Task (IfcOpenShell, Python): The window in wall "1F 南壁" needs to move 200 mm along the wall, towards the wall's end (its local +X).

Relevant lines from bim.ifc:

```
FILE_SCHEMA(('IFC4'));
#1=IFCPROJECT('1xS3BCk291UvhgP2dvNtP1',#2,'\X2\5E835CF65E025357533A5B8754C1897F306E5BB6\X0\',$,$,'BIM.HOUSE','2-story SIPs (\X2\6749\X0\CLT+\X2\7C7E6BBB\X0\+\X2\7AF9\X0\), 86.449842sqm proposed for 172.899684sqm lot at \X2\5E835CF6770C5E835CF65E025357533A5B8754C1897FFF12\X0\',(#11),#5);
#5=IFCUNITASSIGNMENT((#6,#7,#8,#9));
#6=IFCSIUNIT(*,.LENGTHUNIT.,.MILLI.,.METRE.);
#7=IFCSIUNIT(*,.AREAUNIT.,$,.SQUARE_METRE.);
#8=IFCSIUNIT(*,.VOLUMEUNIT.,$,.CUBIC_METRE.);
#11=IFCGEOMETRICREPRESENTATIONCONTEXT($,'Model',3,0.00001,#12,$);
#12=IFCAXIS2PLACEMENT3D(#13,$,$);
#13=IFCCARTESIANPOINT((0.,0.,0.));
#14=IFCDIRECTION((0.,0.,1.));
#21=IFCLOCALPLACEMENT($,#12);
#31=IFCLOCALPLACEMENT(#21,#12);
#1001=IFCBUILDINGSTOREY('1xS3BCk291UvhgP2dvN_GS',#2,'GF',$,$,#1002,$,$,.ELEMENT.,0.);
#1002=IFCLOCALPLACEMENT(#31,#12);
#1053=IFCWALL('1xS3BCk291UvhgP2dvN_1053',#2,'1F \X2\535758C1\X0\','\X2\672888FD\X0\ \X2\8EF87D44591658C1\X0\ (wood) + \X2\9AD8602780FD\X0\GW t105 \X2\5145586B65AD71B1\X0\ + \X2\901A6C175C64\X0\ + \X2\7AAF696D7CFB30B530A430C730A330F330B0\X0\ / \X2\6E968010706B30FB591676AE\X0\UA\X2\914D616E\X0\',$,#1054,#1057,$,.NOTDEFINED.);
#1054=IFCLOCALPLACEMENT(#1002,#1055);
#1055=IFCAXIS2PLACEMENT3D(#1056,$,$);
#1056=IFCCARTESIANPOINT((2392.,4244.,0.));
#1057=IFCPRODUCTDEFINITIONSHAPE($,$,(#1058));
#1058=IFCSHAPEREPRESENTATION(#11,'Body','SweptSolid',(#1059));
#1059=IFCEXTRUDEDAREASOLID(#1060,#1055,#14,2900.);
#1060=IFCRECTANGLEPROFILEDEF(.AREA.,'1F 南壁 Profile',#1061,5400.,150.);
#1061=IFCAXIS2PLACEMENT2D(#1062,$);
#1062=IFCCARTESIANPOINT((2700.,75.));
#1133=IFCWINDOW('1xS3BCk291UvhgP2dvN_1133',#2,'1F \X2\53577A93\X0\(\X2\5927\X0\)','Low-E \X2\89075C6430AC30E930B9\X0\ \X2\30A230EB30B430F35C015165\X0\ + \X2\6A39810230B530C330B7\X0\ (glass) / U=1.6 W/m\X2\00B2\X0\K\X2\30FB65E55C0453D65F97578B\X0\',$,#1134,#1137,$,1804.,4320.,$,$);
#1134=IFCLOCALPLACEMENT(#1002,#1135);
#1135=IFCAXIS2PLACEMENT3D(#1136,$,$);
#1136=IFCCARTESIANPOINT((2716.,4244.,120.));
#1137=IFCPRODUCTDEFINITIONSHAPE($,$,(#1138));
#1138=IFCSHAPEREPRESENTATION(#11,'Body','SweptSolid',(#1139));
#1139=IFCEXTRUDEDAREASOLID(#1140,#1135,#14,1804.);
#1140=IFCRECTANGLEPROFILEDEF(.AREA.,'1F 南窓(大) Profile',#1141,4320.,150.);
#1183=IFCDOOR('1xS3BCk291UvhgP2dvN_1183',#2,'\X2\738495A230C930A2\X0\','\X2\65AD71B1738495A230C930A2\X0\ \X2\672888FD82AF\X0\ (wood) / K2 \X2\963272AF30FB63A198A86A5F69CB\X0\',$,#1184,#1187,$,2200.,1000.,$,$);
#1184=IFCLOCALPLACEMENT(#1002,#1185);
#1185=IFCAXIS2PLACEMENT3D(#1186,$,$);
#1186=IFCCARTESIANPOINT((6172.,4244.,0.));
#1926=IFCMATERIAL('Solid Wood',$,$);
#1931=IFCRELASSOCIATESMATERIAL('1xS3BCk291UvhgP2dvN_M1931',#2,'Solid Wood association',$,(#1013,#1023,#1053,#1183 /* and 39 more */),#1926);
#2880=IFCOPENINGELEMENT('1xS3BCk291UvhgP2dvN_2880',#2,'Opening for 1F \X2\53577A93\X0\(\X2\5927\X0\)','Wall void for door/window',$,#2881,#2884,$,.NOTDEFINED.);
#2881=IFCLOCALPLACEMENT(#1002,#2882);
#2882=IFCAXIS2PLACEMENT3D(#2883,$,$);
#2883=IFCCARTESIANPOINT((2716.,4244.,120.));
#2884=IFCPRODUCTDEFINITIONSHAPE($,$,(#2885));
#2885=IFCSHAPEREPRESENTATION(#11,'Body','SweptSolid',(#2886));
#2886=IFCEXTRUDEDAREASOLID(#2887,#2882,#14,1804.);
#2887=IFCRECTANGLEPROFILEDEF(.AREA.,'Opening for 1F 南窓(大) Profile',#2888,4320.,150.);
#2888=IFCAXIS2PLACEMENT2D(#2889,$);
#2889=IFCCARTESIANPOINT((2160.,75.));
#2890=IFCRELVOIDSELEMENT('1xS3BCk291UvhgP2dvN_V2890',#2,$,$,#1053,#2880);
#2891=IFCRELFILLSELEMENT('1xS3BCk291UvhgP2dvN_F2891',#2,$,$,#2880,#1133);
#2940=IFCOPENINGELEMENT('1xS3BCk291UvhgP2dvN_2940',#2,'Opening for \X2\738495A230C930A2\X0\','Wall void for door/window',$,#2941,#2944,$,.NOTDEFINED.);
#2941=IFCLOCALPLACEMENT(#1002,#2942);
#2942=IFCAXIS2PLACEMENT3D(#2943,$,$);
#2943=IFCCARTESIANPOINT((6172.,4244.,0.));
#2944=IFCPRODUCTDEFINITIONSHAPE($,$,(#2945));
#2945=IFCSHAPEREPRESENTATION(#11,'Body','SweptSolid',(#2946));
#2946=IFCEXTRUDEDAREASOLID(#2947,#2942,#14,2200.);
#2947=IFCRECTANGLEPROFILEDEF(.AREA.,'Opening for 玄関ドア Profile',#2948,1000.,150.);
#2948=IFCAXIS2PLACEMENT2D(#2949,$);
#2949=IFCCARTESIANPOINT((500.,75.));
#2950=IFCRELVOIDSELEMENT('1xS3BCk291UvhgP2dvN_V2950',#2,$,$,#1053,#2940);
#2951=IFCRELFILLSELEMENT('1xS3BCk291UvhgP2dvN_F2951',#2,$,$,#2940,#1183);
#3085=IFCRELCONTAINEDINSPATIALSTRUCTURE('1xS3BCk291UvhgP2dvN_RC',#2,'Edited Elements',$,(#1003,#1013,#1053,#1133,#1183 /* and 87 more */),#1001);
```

```python
import ifcopenshell
import ifcopenshell.api.geometry
import ifcopenshell.util.placement
import ifcopenshell.util.unit

model = ifcopenshell.open("bim.ifc")
unit_scale = ifcopenshell.util.unit.calculate_unit_scale(model)

window = model.by_guid("1xS3BCk291UvhgP2dvN_1133")
opening = window.FillsVoids[0].RelatingOpeningElement
wall = opening.VoidsElements[0].RelatingBuildingElement

wall_matrix = ifcopenshell.util.placement.get_local_placement(wall.ObjectPlacement)
shift = wall_matrix[:3, 0] * 0.2 / unit_scale
before = ifcopenshell.util.placement.get_local_placement(window.ObjectPlacement)[:3, 3].copy()

# The window is not placed relative to its opening, so move both.
for product in (opening, window):
    matrix = ifcopenshell.util.placement.get_local_placement(product.ObjectPlacement)
    matrix[:3, 3] += shift
    ifcopenshell.api.geometry.edit_object_placement(model, product=product, matrix=matrix, is_si=False)

after = ifcopenshell.util.placement.get_local_placement(window.ObjectPlacement)[:3, 3]
print("window moved by", (after - before).round(3) + 0.0)

model.write("bim_rev.ifc")
```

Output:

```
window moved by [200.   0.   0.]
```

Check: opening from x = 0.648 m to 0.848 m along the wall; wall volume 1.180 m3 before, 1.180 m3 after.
